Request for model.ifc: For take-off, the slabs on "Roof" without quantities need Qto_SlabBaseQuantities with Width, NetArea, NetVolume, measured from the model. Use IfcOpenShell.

First a look at what the model holds.

```python
import ifcopenshell
import ifcopenshell.util.element
import ifcopenshell.util.unit

model = ifcopenshell.open("model.ifc")
print(model.schema)
for unit_type in ("LENGTHUNIT", "AREAUNIT", "VOLUMEUNIT"):
    print(unit_type, ifcopenshell.util.unit.calculate_unit_scale(model, unit_type))
storey = next(s for s in model.by_type("IfcBuildingStorey") if s.Name == "Roof")
slabs = [e for e in ifcopenshell.util.element.get_decomposition(storey) if e.is_a("IfcSlab")]
for e in sorted(slabs, key=lambda e: e.id()):
    print(e.id(), e.is_a(), e.Name, list(ifcopenshell.util.element.get_psets(e, qtos_only=True)), sep=" | ")
```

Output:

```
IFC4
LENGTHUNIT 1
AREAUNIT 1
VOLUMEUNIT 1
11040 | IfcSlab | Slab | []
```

```python
import ifcopenshell
import ifcopenshell.api.pset
import ifcopenshell.geom
import ifcopenshell.util.element
import ifcopenshell.util.shape
import ifcopenshell.util.unit

model = ifcopenshell.open("model.ifc")
unit_scale = ifcopenshell.util.unit.calculate_unit_scale(model)
area_scale = ifcopenshell.util.unit.calculate_unit_scale(model, "AREAUNIT")
volume_scale = ifcopenshell.util.unit.calculate_unit_scale(model, "VOLUMEUNIT")
settings = ifcopenshell.geom.settings()

storey = next(s for s in model.by_type("IfcBuildingStorey") if s.Name == "Roof")
slabs = [e for e in ifcopenshell.util.element.get_decomposition(storey) if e.is_a("IfcSlab")]

for e in sorted(slabs, key=lambda e: e.id()):
    if ifcopenshell.util.element.get_psets(e, qtos_only=True, should_inherit=False):
        continue
    # Geometry comes back in metres, in the element's own axes.
    shape = ifcopenshell.geom.create_shape(settings, e)
    values = {
        "Width": ifcopenshell.util.shape.get_z(shape.geometry) / unit_scale,
        "NetArea": ifcopenshell.util.shape.get_footprint_area(shape.geometry) / area_scale,
        "NetVolume": ifcopenshell.util.shape.get_volume(shape.geometry) / volume_scale,
    }
    qto = ifcopenshell.api.pset.add_qto(model, product=e, name="Qto_SlabBaseQuantities")
    ifcopenshell.api.pset.edit_qto(model, qto=qto, properties=values)
    print(e.id(), {k: round(v, 3) for k, v in values.items()})

model.write("model_v2.ifc")
```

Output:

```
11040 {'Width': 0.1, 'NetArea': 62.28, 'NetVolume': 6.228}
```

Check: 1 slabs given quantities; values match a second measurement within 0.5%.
